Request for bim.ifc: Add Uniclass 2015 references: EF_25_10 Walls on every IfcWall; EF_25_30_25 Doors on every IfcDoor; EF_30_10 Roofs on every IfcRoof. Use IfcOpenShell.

First a look at what the model holds.

```python
import ifcopenshell

model = ifcopenshell.open("bim.ifc")
print(model.schema)
print("classifications:", [c.Name for c in model.by_type("IfcClassification")])
for ifc_class in ("IfcDoor", "IfcRoof", "IfcStair", "IfcWall", "IfcWindow"):
    print(ifc_class, len(model.by_type(ifc_class)))
```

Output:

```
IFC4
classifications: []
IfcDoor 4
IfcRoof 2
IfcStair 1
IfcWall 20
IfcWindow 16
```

```python
import ifcopenshell
import ifcopenshell.api.classification

model = ifcopenshell.open("bim.ifc")

system = ifcopenshell.api.classification.add_classification(model, classification="Uniclass 2015")

codes = {
    "IfcWall": ("EF_25_10", "Walls"),
    "IfcDoor": ("EF_25_30_25", "Doors"),
    "IfcRoof": ("EF_30_10", "Roofs"),
}
for ifc_class, (code, name) in codes.items():
    products = model.by_type(ifc_class)
    ifcopenshell.api.classification.add_reference(
        model, products=products, classification=system, identification=code, name=name
    )
    print(code, len(products))

model.write("bim_v2.ifc")
```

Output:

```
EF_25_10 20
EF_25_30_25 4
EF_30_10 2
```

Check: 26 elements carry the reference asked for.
